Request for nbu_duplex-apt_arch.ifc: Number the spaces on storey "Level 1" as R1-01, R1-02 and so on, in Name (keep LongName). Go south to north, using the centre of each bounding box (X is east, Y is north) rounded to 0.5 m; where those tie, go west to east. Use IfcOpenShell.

First a look at what the model holds.

```python
import ifcopenshell
import ifcopenshell.util.element
import ifcopenshell.util.placement

model = ifcopenshell.open("nbu_duplex-apt_arch.ifc")
print(model.schema)
storey = next(s for s in model.by_type("IfcBuildingStorey") if s.Name == "Level 1")
spaces = [e for e in ifcopenshell.util.element.get_decomposition(storey) if e.is_a("IfcSpace")]
for e in sorted(spaces, key=lambda e: e.id()):
    origin = ifcopenshell.util.placement.get_local_placement(e.ObjectPlacement)[:3, 3]
    print(e.id(), e.Name, e.LongName, origin.round(2) + 0.0, sep=" | ")
```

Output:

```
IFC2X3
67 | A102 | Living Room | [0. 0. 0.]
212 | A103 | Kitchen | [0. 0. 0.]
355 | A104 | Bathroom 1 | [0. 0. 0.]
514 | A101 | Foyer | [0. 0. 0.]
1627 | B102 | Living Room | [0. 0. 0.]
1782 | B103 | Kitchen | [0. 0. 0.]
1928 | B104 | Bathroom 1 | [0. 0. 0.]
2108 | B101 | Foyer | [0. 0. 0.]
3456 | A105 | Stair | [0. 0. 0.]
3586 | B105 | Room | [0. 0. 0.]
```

```python
import ifcopenshell
import ifcopenshell.geom
import ifcopenshell.util.element
import ifcopenshell.util.shape

model = ifcopenshell.open("nbu_duplex-apt_arch.ifc")
settings = ifcopenshell.geom.settings()
settings.set("use-world-coords", True)


def centre(element):
    shape = ifcopenshell.geom.create_shape(settings, element)
    return ifcopenshell.util.shape.get_bbox_centroid(shape.geometry)


storey = next(s for s in model.by_type("IfcBuildingStorey") if s.Name == "Level 1")
spaces = [e for e in ifcopenshell.util.element.get_decomposition(storey) if e.is_a("IfcSpace")]

# Insertion points can sit at a corner or the storey origin, so sort by the geometry (in metres).
centres = {e: centre(e) for e in spaces}
spaces.sort(key=lambda e: (round(centres[e][1] / 0.5), centres[e][0]))

for i, e in enumerate(spaces, start=1):
    number = f"R1-{i:02d}"
    e.Name = number
    print(e.id(), number)

model.write("nbu_duplex-apt_arch_edited.ifc")
```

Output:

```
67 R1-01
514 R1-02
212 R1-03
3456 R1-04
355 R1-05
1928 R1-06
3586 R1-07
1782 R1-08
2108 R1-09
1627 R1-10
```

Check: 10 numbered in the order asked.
